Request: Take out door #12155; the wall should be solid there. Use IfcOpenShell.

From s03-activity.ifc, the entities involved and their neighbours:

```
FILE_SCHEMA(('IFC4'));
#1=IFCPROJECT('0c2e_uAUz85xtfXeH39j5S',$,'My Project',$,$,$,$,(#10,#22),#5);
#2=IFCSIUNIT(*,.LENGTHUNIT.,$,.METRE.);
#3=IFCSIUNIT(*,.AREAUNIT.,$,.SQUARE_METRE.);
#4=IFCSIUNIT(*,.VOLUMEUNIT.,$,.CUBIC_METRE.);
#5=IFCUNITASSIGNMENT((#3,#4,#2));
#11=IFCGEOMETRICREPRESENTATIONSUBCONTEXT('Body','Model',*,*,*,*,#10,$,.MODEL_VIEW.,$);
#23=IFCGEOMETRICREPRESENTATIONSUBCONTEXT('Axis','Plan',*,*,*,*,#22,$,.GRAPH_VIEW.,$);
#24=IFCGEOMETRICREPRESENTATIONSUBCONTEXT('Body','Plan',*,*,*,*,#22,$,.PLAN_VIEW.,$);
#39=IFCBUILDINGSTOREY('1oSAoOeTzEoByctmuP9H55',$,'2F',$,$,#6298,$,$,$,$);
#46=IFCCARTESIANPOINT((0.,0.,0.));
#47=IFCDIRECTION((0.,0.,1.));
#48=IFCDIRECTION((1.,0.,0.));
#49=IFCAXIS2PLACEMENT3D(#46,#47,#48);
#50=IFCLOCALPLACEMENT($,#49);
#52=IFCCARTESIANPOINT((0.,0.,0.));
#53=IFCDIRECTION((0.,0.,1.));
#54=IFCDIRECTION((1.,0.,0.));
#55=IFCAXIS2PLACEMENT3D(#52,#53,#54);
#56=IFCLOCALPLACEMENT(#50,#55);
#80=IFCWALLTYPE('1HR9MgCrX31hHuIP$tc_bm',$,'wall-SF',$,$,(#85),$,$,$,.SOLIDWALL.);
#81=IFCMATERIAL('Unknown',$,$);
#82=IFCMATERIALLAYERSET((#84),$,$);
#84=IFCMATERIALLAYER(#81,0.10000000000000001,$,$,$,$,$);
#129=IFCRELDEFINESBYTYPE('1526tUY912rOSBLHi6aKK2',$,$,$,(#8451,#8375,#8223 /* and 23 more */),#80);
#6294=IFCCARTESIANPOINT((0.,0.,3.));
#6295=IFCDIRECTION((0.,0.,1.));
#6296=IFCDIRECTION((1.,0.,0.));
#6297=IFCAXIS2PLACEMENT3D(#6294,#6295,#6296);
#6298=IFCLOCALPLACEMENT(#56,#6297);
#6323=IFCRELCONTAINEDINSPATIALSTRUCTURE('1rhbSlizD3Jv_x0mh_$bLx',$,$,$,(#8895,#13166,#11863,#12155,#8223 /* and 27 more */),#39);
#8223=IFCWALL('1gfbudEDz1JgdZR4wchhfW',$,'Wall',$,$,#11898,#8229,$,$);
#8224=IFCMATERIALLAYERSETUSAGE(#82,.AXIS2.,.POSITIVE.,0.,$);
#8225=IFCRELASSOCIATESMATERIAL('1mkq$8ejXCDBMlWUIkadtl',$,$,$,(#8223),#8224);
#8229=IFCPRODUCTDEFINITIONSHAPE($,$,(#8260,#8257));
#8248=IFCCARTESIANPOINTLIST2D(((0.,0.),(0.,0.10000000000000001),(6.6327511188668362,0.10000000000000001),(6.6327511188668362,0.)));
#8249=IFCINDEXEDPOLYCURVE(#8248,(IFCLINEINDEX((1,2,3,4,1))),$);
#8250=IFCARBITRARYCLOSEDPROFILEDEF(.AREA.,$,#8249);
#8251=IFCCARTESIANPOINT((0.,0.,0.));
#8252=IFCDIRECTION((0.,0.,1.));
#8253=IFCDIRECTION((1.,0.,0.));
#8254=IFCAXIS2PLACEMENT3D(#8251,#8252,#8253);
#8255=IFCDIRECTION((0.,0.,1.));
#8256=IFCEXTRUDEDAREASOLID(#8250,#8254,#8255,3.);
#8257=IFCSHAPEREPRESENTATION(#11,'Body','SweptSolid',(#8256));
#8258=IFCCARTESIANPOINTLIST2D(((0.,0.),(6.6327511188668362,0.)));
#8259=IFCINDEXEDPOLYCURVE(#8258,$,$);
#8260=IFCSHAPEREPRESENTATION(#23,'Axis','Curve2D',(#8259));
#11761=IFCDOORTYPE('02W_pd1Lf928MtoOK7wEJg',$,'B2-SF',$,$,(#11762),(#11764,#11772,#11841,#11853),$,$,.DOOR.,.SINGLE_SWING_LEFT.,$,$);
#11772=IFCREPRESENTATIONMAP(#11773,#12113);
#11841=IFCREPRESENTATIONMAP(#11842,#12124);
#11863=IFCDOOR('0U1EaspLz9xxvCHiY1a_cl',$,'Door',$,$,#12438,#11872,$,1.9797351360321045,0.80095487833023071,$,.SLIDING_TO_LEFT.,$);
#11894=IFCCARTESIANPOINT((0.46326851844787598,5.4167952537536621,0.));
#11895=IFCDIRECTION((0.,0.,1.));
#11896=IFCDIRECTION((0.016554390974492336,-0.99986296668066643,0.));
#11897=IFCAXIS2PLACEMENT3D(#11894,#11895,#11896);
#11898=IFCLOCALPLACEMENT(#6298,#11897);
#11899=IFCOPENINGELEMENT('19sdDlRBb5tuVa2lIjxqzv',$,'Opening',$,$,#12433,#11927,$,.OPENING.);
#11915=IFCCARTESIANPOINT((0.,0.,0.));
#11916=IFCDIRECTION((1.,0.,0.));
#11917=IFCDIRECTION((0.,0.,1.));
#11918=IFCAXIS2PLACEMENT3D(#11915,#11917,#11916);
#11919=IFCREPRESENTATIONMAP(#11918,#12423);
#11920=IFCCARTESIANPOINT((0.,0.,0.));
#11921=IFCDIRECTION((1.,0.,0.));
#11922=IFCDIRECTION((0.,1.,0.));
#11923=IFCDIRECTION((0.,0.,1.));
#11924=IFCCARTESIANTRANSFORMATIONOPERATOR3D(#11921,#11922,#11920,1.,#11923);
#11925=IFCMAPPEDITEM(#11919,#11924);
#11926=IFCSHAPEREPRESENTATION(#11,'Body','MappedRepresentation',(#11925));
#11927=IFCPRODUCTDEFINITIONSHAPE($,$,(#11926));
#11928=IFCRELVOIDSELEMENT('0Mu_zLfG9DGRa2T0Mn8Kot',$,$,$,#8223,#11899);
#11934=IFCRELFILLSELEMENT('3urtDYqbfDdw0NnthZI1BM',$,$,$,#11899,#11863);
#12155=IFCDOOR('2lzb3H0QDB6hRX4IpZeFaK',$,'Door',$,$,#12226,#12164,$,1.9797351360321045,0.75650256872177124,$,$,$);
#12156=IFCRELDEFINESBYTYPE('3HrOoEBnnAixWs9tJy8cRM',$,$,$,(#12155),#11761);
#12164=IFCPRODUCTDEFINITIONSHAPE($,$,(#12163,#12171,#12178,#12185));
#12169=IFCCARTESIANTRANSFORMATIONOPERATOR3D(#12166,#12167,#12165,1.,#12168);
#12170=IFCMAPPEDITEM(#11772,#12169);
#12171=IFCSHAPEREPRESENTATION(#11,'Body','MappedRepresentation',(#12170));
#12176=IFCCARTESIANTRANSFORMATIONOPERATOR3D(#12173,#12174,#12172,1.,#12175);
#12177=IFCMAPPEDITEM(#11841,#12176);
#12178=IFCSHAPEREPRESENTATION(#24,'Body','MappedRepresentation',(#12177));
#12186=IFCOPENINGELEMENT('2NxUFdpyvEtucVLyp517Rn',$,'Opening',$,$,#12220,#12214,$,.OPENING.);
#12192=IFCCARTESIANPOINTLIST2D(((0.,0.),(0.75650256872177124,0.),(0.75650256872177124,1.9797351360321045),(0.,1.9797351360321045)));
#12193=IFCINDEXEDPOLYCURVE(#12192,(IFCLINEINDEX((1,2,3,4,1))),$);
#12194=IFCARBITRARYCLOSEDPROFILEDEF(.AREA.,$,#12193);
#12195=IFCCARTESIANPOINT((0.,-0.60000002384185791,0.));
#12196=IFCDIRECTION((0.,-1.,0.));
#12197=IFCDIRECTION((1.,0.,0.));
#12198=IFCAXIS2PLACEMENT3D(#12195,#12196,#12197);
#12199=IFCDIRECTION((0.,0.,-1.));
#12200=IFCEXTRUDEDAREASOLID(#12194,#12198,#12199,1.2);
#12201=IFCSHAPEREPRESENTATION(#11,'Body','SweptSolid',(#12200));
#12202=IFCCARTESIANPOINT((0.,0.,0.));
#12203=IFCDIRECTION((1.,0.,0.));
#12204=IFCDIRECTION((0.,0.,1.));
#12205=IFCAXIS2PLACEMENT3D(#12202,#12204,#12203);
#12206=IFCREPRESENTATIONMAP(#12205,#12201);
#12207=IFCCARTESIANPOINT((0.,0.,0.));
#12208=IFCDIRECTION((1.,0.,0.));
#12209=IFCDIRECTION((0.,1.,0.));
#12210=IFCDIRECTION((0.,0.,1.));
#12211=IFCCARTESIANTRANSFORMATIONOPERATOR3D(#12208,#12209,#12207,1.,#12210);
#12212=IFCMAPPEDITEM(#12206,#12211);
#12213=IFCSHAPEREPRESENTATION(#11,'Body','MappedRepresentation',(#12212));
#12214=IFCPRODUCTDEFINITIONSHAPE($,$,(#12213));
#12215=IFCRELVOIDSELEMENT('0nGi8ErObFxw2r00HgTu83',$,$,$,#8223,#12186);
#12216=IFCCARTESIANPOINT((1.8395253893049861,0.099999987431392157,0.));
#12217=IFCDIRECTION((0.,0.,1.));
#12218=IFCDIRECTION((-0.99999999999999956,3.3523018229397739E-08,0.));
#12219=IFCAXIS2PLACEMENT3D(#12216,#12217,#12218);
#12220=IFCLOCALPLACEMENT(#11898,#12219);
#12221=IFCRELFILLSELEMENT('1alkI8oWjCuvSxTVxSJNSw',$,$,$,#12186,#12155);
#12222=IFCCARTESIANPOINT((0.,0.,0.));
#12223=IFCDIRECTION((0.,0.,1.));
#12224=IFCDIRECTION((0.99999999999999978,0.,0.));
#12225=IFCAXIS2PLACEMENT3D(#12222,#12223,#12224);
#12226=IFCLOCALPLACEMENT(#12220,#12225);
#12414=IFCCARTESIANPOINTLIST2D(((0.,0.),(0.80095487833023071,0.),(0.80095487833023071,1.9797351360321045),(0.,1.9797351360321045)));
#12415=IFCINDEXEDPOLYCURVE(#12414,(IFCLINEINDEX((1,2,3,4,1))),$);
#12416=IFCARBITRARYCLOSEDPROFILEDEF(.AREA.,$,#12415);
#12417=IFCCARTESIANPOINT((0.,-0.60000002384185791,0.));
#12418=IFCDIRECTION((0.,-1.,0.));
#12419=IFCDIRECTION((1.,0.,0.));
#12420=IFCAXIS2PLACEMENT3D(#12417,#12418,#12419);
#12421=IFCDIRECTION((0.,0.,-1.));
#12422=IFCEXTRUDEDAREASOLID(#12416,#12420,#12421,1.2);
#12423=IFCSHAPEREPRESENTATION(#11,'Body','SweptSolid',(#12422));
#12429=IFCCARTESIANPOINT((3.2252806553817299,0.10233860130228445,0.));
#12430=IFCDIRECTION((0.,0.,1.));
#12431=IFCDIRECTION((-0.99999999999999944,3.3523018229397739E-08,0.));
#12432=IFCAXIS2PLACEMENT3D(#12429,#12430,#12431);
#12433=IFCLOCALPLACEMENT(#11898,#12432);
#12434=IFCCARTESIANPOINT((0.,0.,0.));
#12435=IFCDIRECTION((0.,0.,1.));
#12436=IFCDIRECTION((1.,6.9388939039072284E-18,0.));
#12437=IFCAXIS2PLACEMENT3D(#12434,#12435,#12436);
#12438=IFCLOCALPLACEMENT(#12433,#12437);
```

```python
import ifcopenshell
import ifcopenshell.api.feature
import ifcopenshell.api.root
import ifcopenshell.geom
import ifcopenshell.util.shape

model = ifcopenshell.open("s03-activity.ifc")
settings = ifcopenshell.geom.settings()


def volume(element):
    """Net volume in cubic metres, openings subtracted."""
    shape = ifcopenshell.geom.create_shape(settings, element)
    return ifcopenshell.util.shape.get_volume(shape.geometry)


door = model.by_guid("2lzb3H0QDB6hRX4IpZeFaK")
opening = door.FillsVoids[0].RelatingOpeningElement
wall = opening.VoidsElements[0].RelatingBuildingElement
before = volume(wall)

ifcopenshell.api.root.remove_product(model, product=door)
ifcopenshell.api.feature.remove_feature(model, feature=opening)

after = volume(wall)

print(f"wall volume {before:.3f} -> {after:.3f} m3")

model.write("s03-activity-out.ifc")
```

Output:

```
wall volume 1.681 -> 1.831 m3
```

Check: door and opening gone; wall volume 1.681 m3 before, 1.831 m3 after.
